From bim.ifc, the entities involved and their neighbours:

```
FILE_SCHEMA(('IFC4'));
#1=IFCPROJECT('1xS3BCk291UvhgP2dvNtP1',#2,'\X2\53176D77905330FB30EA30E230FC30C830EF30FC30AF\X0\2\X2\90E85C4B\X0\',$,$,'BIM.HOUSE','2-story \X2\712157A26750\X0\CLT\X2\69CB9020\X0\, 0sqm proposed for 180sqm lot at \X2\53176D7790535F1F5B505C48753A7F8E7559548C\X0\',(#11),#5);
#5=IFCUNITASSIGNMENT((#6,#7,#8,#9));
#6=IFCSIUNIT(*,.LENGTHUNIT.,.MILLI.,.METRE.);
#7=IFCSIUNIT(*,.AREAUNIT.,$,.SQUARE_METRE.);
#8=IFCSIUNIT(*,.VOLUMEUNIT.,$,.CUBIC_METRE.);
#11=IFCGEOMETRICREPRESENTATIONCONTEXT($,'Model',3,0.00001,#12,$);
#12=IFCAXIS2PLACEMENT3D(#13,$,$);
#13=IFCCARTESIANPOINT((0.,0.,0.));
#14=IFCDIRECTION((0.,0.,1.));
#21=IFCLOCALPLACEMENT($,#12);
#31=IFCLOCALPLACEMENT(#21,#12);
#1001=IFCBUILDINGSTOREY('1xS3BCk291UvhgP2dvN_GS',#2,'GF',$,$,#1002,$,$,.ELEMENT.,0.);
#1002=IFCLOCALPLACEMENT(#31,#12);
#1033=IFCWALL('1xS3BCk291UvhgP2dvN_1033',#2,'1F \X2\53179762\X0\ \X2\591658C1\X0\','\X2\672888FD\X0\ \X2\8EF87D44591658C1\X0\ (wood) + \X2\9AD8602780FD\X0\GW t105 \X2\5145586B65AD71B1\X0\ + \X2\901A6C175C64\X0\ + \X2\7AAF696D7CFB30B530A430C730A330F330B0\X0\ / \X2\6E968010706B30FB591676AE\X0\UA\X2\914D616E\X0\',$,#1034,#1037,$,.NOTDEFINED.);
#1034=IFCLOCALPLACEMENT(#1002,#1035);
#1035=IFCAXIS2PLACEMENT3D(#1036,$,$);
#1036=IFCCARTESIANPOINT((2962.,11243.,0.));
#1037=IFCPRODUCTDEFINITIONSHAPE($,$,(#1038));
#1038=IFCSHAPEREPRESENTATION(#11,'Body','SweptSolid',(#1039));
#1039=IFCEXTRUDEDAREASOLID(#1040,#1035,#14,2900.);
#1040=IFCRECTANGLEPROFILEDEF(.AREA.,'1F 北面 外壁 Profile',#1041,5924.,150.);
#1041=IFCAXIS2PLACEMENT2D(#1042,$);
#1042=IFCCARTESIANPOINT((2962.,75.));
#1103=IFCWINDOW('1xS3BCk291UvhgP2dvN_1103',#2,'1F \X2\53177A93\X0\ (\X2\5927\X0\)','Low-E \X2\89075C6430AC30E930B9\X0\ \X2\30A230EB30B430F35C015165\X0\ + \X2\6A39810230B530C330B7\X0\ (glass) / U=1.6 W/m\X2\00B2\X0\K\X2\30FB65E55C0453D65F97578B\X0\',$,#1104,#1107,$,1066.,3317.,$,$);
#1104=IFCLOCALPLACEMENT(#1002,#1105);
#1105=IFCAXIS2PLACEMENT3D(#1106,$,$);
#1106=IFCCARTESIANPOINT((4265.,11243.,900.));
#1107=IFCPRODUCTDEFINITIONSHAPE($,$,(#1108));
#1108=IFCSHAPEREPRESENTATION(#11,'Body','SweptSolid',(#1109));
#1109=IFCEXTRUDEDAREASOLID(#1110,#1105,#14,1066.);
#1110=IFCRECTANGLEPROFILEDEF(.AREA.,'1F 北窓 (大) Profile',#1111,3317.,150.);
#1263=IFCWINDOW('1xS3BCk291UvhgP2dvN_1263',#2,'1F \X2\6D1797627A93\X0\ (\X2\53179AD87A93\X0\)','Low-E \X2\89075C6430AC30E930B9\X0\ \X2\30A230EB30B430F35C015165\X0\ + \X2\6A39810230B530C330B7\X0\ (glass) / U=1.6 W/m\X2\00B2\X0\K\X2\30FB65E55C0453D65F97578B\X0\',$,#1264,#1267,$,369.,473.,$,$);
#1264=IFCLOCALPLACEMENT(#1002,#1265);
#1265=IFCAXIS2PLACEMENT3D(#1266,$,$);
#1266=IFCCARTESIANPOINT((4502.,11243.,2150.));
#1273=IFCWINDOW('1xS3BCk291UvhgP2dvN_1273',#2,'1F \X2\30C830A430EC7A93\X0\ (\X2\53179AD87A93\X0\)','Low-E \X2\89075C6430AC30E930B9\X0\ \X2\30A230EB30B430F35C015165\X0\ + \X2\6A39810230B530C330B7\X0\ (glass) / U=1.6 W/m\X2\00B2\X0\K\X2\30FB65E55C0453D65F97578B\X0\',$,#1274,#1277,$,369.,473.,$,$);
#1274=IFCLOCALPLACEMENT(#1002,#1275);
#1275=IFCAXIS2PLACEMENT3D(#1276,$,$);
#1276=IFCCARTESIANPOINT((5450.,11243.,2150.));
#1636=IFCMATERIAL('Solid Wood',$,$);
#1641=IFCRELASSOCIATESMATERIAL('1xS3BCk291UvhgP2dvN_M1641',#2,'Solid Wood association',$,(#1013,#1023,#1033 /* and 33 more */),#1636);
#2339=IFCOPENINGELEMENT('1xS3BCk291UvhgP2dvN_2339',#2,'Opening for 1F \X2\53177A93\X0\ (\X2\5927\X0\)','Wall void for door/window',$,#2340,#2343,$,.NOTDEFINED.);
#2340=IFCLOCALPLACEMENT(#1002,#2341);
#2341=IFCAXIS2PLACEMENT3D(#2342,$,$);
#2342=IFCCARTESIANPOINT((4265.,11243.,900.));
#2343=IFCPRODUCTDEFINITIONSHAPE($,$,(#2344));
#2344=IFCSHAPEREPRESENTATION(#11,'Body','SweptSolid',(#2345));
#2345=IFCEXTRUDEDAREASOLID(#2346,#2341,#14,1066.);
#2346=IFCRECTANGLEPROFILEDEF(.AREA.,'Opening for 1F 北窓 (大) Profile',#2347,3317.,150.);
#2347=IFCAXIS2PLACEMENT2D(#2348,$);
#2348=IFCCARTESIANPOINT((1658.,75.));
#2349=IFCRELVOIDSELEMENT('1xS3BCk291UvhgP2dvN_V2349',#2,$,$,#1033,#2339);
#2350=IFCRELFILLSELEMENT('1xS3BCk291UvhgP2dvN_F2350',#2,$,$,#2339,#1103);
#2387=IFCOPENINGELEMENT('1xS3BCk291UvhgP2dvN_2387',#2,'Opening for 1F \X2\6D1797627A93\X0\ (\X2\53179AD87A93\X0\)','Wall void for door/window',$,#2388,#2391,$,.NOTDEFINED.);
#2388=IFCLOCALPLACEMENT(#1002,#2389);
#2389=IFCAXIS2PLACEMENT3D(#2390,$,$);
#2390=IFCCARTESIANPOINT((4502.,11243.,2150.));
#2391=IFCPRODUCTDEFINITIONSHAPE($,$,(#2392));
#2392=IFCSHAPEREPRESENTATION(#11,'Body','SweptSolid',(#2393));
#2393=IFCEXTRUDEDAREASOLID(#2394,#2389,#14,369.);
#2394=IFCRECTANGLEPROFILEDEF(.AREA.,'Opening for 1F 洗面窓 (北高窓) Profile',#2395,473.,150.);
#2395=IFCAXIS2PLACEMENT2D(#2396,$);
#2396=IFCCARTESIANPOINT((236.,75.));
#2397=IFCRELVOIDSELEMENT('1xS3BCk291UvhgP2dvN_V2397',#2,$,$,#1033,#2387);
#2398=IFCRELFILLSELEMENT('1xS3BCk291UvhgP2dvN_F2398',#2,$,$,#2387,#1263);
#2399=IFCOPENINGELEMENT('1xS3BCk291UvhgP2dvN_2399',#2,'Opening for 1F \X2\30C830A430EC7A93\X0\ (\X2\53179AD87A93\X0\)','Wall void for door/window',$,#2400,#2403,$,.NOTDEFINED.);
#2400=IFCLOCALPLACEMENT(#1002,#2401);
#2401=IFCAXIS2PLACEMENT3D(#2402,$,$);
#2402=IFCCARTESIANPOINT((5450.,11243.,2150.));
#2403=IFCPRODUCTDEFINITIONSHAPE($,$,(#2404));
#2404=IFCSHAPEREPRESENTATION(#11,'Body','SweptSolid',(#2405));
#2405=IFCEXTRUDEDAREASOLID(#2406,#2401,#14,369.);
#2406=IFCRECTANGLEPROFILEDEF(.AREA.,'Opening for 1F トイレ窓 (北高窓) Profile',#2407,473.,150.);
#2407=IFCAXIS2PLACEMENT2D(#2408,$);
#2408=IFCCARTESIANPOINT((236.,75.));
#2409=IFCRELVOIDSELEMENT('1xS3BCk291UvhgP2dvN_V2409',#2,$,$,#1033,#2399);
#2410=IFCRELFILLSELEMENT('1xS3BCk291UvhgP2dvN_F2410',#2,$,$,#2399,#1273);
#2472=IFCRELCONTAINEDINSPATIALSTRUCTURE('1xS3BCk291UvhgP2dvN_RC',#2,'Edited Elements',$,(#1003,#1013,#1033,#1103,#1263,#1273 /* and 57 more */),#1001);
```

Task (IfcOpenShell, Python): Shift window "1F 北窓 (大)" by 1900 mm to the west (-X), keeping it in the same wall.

```python
import ifcopenshell
import ifcopenshell.api.geometry
import ifcopenshell.util.placement

model = ifcopenshell.open("bim.ifc")

window = model.by_guid("1xS3BCk291UvhgP2dvN_1103")
opening = window.FillsVoids[0].RelatingOpeningElement
wall = opening.VoidsElements[0].RelatingBuildingElement

wall_matrix = ifcopenshell.util.placement.get_local_placement(wall.ObjectPlacement)
shift = wall_matrix[:3, 0] * -1900.0
before = ifcopenshell.util.placement.get_local_placement(window.ObjectPlacement)[:3, 3].copy()

# The window is not placed relative to its opening, so move both.
for product in (opening, window):
    matrix = ifcopenshell.util.placement.get_local_placement(product.ObjectPlacement)
    matrix[:3, 3] += shift
    ifcopenshell.api.geometry.edit_object_placement(model, product=product, matrix=matrix, is_si=False)

after = ifcopenshell.util.placement.get_local_placement(window.ObjectPlacement)[:3, 3]
print("window moved by", (after - before).round(3) + 0.0)

model.write("bim_v2.ifc")
```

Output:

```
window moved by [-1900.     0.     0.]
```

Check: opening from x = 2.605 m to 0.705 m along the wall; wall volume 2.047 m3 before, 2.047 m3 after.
